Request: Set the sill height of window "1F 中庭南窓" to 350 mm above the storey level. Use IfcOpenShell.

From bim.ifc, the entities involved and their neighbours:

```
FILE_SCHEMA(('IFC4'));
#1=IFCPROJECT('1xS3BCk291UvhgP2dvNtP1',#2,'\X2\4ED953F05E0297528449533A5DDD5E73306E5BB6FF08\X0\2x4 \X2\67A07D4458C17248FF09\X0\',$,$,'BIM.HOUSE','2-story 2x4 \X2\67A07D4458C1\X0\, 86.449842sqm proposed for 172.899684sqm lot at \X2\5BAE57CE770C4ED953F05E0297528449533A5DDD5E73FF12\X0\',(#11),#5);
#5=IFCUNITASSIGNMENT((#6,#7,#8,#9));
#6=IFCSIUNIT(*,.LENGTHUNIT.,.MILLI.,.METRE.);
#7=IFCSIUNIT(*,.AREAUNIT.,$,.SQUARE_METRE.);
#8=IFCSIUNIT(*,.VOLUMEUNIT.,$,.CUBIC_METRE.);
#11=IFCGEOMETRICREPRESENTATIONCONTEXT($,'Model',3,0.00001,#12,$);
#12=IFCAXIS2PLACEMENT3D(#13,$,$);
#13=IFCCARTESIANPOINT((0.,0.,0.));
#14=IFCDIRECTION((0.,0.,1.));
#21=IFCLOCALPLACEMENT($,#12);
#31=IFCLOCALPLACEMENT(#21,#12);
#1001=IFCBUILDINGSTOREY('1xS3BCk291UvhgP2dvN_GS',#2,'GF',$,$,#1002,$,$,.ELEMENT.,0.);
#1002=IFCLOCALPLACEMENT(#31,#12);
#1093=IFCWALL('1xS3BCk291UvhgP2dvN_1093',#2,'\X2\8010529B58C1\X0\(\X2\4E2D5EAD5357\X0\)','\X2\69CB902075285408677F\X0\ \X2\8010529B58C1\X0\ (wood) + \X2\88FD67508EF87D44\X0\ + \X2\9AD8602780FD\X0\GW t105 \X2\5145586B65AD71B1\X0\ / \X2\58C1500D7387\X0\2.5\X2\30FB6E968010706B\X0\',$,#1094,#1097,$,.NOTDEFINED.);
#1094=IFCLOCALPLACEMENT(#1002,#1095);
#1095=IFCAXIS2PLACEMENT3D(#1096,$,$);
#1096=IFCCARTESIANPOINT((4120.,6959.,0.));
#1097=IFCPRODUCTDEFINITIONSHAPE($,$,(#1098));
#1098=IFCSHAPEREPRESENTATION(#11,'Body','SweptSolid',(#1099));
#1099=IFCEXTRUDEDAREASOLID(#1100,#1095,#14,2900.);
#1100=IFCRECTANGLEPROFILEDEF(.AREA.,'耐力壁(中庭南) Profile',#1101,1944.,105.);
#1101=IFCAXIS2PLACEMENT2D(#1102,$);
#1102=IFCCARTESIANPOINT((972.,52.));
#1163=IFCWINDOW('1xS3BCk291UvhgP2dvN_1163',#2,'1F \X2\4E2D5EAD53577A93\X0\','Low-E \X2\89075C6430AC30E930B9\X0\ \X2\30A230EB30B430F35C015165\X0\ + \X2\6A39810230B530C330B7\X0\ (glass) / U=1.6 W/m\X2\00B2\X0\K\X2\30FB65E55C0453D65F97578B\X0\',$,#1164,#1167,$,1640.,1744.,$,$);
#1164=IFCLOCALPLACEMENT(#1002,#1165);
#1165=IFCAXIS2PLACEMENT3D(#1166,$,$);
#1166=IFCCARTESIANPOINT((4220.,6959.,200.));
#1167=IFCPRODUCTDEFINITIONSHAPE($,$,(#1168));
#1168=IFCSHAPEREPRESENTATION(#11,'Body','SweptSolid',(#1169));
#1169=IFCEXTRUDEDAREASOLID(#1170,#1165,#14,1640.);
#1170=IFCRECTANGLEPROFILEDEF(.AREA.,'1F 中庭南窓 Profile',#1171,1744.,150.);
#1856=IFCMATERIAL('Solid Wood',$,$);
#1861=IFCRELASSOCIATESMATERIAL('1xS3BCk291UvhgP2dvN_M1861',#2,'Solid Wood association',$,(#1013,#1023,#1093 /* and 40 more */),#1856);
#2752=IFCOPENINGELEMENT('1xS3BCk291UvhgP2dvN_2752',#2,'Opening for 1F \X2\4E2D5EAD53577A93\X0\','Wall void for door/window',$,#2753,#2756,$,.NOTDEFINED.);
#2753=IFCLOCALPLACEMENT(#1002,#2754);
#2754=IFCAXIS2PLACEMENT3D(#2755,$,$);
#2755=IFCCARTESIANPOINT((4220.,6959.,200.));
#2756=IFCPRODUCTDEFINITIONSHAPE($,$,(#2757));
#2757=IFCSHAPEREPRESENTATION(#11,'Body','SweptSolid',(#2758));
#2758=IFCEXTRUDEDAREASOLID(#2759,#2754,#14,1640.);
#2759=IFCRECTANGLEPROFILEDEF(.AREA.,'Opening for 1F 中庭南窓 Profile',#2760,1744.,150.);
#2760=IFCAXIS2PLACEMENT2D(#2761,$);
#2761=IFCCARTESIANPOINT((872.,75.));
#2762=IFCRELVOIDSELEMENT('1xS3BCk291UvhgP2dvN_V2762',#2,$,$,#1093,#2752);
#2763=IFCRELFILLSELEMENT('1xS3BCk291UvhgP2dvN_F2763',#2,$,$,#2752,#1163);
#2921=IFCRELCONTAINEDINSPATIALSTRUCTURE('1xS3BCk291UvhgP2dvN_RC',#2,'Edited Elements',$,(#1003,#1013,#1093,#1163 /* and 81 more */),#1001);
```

```python
import numpy as np
import ifcopenshell
import ifcopenshell.api.geometry
import ifcopenshell.geom
import ifcopenshell.util.element
import ifcopenshell.util.placement
import ifcopenshell.util.shape
import ifcopenshell.util.unit

model = ifcopenshell.open("bim.ifc")
unit_scale = ifcopenshell.util.unit.calculate_unit_scale(model)

window = model.by_guid("1xS3BCk291UvhgP2dvN_1163")
opening = window.FillsVoids[0].RelatingOpeningElement
storey = ifcopenshell.util.element.get_container(window, ifc_class="IfcBuildingStorey")
level = ifcopenshell.util.placement.get_local_placement(storey.ObjectPlacement)[2, 3]

# The opening's origin need not be at the sill, so measure its lowest point.
shape = ifcopenshell.geom.create_shape(ifcopenshell.geom.settings(), opening)
bottom = ifcopenshell.util.shape.get_shape_bottom_elevation(shape, shape.geometry) / unit_scale
dz = level + 0.35 / unit_scale - bottom

shift = np.array([0.0, 0.0, dz])
# The window is not placed relative to its opening, so move both.
for product in (opening, window):
    matrix = ifcopenshell.util.placement.get_local_placement(product.ObjectPlacement)
    matrix[:3, 3] += shift
    ifcopenshell.api.geometry.edit_object_placement(model, product=product, matrix=matrix, is_si=False)

print(f"moved by {dz * unit_scale:+.3f} m")

model.write("bim_updated.ifc")
```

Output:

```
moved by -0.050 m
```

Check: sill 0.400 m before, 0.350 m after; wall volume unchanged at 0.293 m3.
